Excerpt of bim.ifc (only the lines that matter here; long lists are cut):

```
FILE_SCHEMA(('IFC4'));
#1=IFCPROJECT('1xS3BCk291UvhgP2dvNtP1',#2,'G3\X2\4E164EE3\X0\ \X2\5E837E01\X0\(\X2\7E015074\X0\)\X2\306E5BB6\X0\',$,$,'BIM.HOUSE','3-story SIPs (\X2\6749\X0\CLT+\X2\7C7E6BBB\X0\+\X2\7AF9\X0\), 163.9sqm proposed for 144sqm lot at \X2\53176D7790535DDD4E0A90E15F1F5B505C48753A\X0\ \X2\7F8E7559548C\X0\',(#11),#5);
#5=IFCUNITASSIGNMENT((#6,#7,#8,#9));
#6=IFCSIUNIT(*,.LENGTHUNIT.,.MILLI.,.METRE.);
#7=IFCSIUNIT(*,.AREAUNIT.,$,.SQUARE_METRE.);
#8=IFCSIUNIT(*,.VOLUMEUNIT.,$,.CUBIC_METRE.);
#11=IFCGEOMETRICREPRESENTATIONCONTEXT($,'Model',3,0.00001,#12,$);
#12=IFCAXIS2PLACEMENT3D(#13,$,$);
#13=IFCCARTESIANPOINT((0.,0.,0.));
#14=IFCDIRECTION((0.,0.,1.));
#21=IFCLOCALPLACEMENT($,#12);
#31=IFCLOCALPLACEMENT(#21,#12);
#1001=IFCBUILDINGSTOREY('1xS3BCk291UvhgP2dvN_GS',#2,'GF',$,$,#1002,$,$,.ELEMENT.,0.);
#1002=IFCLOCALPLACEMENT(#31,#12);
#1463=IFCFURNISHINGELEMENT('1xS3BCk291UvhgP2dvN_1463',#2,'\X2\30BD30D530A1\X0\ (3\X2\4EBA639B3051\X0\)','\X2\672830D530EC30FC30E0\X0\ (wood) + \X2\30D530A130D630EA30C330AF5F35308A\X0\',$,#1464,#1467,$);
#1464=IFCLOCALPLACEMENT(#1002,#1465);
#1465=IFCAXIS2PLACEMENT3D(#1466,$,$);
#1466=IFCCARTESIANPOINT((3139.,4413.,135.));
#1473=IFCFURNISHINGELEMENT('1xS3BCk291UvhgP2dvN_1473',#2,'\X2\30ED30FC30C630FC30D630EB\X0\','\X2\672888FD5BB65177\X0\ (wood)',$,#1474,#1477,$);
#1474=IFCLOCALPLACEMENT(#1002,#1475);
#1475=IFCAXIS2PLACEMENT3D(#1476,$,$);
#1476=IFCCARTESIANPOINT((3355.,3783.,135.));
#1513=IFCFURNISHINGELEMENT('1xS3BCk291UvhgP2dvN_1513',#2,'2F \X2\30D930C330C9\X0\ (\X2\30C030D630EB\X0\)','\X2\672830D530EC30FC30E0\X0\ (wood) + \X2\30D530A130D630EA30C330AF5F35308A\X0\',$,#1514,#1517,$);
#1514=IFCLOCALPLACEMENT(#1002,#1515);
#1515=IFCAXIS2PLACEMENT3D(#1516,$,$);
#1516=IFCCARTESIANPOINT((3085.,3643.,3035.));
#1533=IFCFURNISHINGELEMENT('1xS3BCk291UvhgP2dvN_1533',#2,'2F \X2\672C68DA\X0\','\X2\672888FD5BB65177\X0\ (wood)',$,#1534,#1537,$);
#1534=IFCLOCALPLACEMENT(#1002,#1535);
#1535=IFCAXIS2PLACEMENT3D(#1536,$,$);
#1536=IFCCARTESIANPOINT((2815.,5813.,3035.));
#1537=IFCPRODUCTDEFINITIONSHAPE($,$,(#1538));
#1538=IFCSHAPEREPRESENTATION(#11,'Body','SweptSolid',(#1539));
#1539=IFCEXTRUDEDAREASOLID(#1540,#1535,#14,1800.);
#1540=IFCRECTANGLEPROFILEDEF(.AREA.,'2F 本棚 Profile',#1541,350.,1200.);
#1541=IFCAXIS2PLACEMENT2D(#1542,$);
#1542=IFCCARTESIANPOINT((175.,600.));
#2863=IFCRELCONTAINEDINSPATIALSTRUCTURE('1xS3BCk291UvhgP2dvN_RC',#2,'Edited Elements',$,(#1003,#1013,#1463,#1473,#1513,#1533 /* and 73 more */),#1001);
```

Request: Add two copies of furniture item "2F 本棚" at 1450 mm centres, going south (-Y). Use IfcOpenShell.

```python
import numpy as np
import ifcopenshell
import ifcopenshell.api.geometry
import ifcopenshell.api.root
import ifcopenshell.util.element
import ifcopenshell.util.placement
import ifcopenshell.util.unit

model = ifcopenshell.open("bim.ifc")
unit_scale = ifcopenshell.util.unit.calculate_unit_scale(model)


def reuse_history(source, copy):
    """copy_class also copies each property set's owner history, people and application; keep the originals."""
    for rel in copy.IsDefinedBy:
        if rel.is_a("IfcRelDefinesByProperties") and (history := rel.RelatingPropertyDefinition.OwnerHistory):
            rel.RelatingPropertyDefinition.OwnerHistory = source.OwnerHistory
            ifcopenshell.util.element.remove_deep2(model, history)


source = model.by_id(1533)
base = ifcopenshell.util.placement.get_local_placement(source.ObjectPlacement)
step = np.array([0.0, -1.0, 0.0]) * 1.45 / unit_scale

for i in range(1, 3):
    copy = ifcopenshell.api.root.copy_class(model, product=source)
    copy.Representation = ifcopenshell.util.element.copy_deep(
        model, source.Representation, exclude=["IfcGeometricRepresentationContext", "IfcRepresentationMap"]
    )
    reuse_history(source, copy)
    matrix = base.copy()
    matrix[:3, 3] += i * step
    print("added at", matrix[:3, 3].round(3) + 0.0)
    ifcopenshell.api.geometry.edit_object_placement(model, product=copy, matrix=matrix, is_si=False)

model.write("bim_rev.ifc")
```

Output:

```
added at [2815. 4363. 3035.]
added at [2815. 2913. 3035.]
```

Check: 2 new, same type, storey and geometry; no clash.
